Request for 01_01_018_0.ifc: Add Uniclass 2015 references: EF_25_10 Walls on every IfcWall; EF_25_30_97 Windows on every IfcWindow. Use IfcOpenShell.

First a look at what the model holds.

```python
import ifcopenshell

model = ifcopenshell.open("01_01_018_0.ifc")
print(model.schema)
print("classifications:", [c.Name for c in model.by_type("IfcClassification")])
for ifc_class in ("IfcDoor", "IfcRoof", "IfcStair", "IfcWall", "IfcWindow"):
    print(ifc_class, len(model.by_type(ifc_class)))
```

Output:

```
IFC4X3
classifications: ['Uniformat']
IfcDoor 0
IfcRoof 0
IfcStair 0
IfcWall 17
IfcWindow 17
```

```python
import ifcopenshell
import ifcopenshell.api.classification

model = ifcopenshell.open("01_01_018_0.ifc")

system = ifcopenshell.api.classification.add_classification(model, classification="Uniclass 2015")

codes = {
    "IfcWall": ("EF_25_10", "Walls"),
    "IfcWindow": ("EF_25_30_97", "Windows"),
}
for ifc_class, (code, name) in codes.items():
    products = model.by_type(ifc_class)
    ifcopenshell.api.classification.add_reference(
        model, products=products, classification=system, identification=code, name=name
    )
    print(code, len(products))

model.write("01_01_018_0_v2.ifc")
```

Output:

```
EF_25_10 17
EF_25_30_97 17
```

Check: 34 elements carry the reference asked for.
